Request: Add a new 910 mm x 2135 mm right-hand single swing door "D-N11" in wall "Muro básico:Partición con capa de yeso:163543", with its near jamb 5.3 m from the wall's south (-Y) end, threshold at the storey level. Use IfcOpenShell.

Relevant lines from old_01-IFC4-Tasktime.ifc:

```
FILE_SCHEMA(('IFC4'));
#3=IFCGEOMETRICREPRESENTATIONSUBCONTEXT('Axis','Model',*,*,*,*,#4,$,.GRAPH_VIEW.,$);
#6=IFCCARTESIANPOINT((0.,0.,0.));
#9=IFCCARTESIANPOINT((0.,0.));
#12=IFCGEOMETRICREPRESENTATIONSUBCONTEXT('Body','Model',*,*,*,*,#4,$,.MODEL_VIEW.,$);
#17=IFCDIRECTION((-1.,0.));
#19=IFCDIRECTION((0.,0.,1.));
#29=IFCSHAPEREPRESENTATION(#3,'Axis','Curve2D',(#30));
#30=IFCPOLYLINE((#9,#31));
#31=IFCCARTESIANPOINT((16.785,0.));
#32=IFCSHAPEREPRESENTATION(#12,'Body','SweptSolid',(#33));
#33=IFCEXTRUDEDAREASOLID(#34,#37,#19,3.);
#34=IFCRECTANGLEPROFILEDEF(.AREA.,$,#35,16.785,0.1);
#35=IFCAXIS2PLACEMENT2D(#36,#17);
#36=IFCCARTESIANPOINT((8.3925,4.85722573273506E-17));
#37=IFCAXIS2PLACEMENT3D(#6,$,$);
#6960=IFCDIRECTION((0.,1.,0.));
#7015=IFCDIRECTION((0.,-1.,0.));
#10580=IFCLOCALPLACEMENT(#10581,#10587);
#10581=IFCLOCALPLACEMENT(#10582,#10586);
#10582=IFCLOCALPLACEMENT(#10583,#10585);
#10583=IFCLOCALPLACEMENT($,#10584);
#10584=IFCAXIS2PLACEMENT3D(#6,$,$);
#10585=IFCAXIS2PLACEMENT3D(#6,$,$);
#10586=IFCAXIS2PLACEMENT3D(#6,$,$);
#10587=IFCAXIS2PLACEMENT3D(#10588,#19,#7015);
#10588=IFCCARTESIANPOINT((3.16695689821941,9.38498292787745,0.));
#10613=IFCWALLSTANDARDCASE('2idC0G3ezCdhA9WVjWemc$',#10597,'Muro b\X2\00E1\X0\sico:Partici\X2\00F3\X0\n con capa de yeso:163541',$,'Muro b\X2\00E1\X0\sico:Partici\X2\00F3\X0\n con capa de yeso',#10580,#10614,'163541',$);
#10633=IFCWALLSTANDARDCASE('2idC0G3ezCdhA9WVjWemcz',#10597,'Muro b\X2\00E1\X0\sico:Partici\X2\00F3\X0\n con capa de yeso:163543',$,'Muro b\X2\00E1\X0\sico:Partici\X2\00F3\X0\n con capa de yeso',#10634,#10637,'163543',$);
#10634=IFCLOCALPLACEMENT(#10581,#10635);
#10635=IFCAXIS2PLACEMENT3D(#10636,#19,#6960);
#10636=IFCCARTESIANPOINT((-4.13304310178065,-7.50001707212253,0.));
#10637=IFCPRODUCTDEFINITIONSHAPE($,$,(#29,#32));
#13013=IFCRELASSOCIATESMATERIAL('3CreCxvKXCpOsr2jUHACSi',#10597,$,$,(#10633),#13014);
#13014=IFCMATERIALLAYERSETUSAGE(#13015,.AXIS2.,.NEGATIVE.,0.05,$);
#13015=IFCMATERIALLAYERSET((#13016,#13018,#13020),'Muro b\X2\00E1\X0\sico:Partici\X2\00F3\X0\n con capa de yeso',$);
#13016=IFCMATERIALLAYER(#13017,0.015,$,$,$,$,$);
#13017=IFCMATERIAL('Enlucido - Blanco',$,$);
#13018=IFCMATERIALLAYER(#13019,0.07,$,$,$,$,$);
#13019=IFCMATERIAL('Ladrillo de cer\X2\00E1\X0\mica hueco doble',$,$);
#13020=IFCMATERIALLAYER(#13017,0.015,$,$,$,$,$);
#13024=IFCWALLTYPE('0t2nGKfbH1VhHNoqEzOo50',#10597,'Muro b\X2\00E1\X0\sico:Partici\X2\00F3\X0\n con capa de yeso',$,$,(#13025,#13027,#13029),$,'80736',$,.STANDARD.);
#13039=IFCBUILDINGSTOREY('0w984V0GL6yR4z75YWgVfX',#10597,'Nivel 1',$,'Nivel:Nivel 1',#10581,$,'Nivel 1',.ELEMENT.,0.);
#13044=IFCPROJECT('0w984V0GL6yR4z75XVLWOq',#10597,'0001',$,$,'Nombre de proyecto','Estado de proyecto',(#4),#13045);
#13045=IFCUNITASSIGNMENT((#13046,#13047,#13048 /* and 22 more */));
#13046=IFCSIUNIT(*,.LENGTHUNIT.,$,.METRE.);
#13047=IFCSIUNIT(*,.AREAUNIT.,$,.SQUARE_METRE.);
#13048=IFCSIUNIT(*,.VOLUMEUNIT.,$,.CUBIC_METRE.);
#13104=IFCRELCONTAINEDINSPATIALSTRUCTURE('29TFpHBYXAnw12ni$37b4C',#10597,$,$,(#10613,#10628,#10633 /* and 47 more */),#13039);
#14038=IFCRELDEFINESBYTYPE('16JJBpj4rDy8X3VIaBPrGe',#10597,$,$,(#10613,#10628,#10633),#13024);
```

```python
import numpy as np
import ifcopenshell
import ifcopenshell.api.feature
import ifcopenshell.api.geometry
import ifcopenshell.api.root
import ifcopenshell.api.spatial
import ifcopenshell.geom
import ifcopenshell.util.element
import ifcopenshell.util.placement
import ifcopenshell.util.representation
import ifcopenshell.util.shape
import ifcopenshell.util.unit

model = ifcopenshell.open("old_01-IFC4-Tasktime.ifc")
unit_scale = ifcopenshell.util.unit.calculate_unit_scale(model)
settings = ifcopenshell.geom.settings()


def volume(element):
    """Net volume in cubic metres, openings subtracted."""
    shape = ifcopenshell.geom.create_shape(settings, element)
    return ifcopenshell.util.shape.get_volume(shape.geometry)


wall = model.by_guid("2idC0G3ezCdhA9WVjWemcz")
storey = ifcopenshell.util.element.get_container(wall, ifc_class="IfcBuildingStorey")
context = ifcopenshell.util.representation.get_context(model, "Model", "Body", "MODEL_VIEW")
before = volume(wall)

width, height, from_end, sill = 0.91, 2.135, 5.3, 0.0  # metres

# The wall runs along its own X axis, and the end named is its -X end.
wall_shape = ifcopenshell.geom.create_shape(settings, wall)
x, y, z = ifcopenshell.util.shape.get_vertices(wall_shape.geometry).T
start = x.min() + from_end
face, thickness = float(y.min()), float(y.max() - y.min())
wall_matrix = ifcopenshell.util.placement.get_local_placement(wall.ObjectPlacement)
level = ifcopenshell.util.placement.get_local_placement(storey.ObjectPlacement)[2, 3]


def in_wall(x, y):
    """Placement at x, y metres in the wall's axes, at sill height."""
    matrix = wall_matrix.copy()
    matrix[:, 3] = wall_matrix @ np.array([x / unit_scale, y / unit_scale, 0.0, 1.0])
    matrix[2, 3] = level + sill / unit_scale
    return matrix


# Opening: a box that overshoots both wall faces by 50 mm.
opening = ifcopenshell.api.root.create_entity(model, ifc_class="IfcOpeningElement", predefined_type="OPENING")
box = ifcopenshell.api.geometry.add_wall_representation(
    model, context=context, length=width, height=height, thickness=thickness + 0.1
)
ifcopenshell.api.geometry.assign_representation(model, product=opening, representation=box)
ifcopenshell.api.geometry.edit_object_placement(model, product=opening, matrix=in_wall(start, face - 0.05), is_si=False)
ifcopenshell.api.feature.add_feature(model, feature=opening, element=wall)

door = ifcopenshell.api.root.create_entity(model, ifc_class="IfcDoor", name="D-N11", predefined_type="DOOR")
door.OverallWidth, door.OverallHeight = width / unit_scale, height / unit_scale
door.OperationType = "SINGLE_SWING_RIGHT"
body = ifcopenshell.api.geometry.add_door_representation(
    model,
    context=context,
    overall_width=door.OverallWidth,
    overall_height=door.OverallHeight,
    operation_type="SINGLE_SWING_RIGHT",
    lining_properties={"LiningDepth": thickness / unit_scale, "ThresholdDepth": thickness / unit_scale},
)
ifcopenshell.api.geometry.assign_representation(model, product=door, representation=body)
ifcopenshell.api.spatial.assign_container(model, products=[door], relating_structure=storey)
ifcopenshell.api.feature.add_filling(model, opening=opening, element=door)

# The lining spans the wall, so the door starts at the wall face.
ifcopenshell.api.geometry.edit_object_placement(model, product=door, matrix=in_wall(start, face), is_si=False)

after = volume(wall)

print(f"wall volume {before:.3f} -> {after:.3f} m3")

model.write("old_01-IFC4-Tasktime_rev.ifc")
```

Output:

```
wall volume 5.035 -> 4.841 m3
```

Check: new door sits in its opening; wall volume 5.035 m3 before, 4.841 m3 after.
